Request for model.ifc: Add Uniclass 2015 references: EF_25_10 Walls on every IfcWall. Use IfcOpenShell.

First a look at what the model holds.

```python
import ifcopenshell

model = ifcopenshell.open("model.ifc")
print(model.schema)
print("classifications:", [c.Name for c in model.by_type("IfcClassification")])
for ifc_class in ("IfcDoor", "IfcRoof", "IfcStair", "IfcWall", "IfcWindow"):
    print(ifc_class, len(model.by_type(ifc_class)))
```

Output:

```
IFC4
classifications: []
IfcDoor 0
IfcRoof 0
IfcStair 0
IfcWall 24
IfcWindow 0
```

```python
import ifcopenshell
import ifcopenshell.api.classification

model = ifcopenshell.open("model.ifc")

system = ifcopenshell.api.classification.add_classification(model, classification="Uniclass 2015")

codes = {
    "IfcWall": ("EF_25_10", "Walls"),
}
for ifc_class, (code, name) in codes.items():
    products = model.by_type(ifc_class)
    ifcopenshell.api.classification.add_reference(
        model, products=products, classification=system, identification=code, name=name
    )
    print(code, len(products))

model.write("model-out.ifc")
```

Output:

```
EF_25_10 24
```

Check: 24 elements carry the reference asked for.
